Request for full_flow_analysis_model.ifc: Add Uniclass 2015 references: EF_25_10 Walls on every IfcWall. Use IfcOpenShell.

First a look at what the model holds.

```python
import ifcopenshell

model = ifcopenshell.open("full_flow_analysis_model.ifc")
print(model.schema)
print("classifications:", [c.Name for c in model.by_type("IfcClassification")])
for ifc_class in ("IfcDoor", "IfcRoof", "IfcStair", "IfcWall", "IfcWindow"):
    print(ifc_class, len(model.by_type(ifc_class)))
```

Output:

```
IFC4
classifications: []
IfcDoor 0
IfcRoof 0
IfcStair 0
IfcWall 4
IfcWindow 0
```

```python
import ifcopenshell
import ifcopenshell.api.classification

model = ifcopenshell.open("full_flow_analysis_model.ifc")

system = ifcopenshell.api.classification.add_classification(model, classification="Uniclass 2015")

codes = {
    "IfcWall": ("EF_25_10", "Walls"),
}
for ifc_class, (code, name) in codes.items():
    products = model.by_type(ifc_class)
    ifcopenshell.api.classification.add_reference(
        model, products=products, classification=system, identification=code, name=name
    )
    print(code, len(products))

model.write("full_flow_analysis_model_rev.ifc")
```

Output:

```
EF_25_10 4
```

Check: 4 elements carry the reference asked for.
